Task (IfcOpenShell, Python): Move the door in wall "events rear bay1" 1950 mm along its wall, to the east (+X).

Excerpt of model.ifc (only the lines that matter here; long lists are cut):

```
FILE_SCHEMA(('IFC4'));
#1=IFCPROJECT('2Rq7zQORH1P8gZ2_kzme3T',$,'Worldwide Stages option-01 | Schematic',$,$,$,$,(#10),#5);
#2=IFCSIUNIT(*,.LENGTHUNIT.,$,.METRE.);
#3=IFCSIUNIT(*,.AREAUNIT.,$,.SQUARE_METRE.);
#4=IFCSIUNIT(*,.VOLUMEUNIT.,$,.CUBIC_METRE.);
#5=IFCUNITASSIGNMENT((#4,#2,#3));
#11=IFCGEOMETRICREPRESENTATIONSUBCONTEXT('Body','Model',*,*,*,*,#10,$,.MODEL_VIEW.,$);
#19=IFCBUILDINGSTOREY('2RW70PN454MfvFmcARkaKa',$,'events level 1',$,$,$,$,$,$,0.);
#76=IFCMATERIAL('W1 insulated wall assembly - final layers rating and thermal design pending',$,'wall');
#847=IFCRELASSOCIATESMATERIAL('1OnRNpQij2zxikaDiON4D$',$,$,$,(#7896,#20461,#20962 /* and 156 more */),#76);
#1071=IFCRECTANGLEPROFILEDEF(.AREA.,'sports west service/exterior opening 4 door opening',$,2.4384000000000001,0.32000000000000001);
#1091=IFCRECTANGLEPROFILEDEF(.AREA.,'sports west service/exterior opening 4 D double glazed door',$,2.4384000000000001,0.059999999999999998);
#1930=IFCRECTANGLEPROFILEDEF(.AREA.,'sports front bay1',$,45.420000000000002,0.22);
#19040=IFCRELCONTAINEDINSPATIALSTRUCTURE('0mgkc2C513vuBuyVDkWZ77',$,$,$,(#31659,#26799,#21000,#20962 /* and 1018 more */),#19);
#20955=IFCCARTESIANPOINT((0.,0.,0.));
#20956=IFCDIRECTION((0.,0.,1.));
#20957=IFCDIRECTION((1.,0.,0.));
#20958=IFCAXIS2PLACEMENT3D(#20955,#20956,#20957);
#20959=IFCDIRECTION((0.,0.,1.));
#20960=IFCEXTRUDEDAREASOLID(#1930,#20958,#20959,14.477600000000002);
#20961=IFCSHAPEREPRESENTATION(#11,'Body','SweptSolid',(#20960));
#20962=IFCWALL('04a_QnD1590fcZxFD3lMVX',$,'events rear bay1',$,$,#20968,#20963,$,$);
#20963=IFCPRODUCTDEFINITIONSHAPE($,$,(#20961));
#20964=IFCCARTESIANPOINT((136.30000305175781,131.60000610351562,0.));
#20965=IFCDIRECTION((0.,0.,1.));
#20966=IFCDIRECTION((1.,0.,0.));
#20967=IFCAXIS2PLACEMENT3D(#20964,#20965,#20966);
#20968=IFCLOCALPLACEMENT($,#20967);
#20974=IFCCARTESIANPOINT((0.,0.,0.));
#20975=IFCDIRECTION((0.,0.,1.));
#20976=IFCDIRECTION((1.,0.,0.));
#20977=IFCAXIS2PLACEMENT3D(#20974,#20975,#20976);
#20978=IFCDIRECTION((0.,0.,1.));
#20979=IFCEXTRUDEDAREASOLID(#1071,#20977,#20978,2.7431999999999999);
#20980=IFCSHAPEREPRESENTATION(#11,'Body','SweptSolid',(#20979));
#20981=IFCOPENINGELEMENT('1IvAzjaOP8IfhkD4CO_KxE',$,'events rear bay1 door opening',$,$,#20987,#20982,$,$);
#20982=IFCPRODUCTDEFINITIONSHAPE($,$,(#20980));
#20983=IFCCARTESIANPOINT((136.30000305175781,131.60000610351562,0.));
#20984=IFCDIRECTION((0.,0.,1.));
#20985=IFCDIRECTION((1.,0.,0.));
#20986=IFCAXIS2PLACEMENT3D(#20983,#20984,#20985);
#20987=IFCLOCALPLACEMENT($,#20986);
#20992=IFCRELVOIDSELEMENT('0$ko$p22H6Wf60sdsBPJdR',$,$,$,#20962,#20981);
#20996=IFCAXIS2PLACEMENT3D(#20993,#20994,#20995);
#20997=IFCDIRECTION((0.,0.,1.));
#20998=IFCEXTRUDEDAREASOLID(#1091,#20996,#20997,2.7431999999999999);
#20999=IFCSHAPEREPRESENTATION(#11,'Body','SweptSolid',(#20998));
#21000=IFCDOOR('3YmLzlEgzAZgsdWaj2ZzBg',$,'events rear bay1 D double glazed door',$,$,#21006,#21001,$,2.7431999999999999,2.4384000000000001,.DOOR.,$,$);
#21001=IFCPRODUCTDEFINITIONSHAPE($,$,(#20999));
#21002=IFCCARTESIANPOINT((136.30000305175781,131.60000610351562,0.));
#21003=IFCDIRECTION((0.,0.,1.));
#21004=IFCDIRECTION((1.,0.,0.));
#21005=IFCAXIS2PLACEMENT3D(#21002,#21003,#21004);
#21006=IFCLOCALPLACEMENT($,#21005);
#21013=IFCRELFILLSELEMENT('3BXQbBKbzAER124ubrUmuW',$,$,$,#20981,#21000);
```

```python
import ifcopenshell
import ifcopenshell.api.geometry
import ifcopenshell.util.placement

model = ifcopenshell.open("model.ifc")

door = model.by_guid("3YmLzlEgzAZgsdWaj2ZzBg")
opening = door.FillsVoids[0].RelatingOpeningElement
wall = opening.VoidsElements[0].RelatingBuildingElement

wall_matrix = ifcopenshell.util.placement.get_local_placement(wall.ObjectPlacement)
shift = wall_matrix[:3, 0] * 1.95
before = ifcopenshell.util.placement.get_local_placement(door.ObjectPlacement)[:3, 3].copy()

# The door is not placed relative to its opening, so move both.
for product in (opening, door):
    matrix = ifcopenshell.util.placement.get_local_placement(product.ObjectPlacement)
    matrix[:3, 3] += shift
    ifcopenshell.api.geometry.edit_object_placement(model, product=product, matrix=matrix, is_si=False)

after = ifcopenshell.util.placement.get_local_placement(door.ObjectPlacement)[:3, 3]
print("door moved by", (after - before).round(3) + 0.0)

model.write("model_edited.ifc")
```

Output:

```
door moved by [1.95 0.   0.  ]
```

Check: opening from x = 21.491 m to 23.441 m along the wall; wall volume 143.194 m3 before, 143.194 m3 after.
